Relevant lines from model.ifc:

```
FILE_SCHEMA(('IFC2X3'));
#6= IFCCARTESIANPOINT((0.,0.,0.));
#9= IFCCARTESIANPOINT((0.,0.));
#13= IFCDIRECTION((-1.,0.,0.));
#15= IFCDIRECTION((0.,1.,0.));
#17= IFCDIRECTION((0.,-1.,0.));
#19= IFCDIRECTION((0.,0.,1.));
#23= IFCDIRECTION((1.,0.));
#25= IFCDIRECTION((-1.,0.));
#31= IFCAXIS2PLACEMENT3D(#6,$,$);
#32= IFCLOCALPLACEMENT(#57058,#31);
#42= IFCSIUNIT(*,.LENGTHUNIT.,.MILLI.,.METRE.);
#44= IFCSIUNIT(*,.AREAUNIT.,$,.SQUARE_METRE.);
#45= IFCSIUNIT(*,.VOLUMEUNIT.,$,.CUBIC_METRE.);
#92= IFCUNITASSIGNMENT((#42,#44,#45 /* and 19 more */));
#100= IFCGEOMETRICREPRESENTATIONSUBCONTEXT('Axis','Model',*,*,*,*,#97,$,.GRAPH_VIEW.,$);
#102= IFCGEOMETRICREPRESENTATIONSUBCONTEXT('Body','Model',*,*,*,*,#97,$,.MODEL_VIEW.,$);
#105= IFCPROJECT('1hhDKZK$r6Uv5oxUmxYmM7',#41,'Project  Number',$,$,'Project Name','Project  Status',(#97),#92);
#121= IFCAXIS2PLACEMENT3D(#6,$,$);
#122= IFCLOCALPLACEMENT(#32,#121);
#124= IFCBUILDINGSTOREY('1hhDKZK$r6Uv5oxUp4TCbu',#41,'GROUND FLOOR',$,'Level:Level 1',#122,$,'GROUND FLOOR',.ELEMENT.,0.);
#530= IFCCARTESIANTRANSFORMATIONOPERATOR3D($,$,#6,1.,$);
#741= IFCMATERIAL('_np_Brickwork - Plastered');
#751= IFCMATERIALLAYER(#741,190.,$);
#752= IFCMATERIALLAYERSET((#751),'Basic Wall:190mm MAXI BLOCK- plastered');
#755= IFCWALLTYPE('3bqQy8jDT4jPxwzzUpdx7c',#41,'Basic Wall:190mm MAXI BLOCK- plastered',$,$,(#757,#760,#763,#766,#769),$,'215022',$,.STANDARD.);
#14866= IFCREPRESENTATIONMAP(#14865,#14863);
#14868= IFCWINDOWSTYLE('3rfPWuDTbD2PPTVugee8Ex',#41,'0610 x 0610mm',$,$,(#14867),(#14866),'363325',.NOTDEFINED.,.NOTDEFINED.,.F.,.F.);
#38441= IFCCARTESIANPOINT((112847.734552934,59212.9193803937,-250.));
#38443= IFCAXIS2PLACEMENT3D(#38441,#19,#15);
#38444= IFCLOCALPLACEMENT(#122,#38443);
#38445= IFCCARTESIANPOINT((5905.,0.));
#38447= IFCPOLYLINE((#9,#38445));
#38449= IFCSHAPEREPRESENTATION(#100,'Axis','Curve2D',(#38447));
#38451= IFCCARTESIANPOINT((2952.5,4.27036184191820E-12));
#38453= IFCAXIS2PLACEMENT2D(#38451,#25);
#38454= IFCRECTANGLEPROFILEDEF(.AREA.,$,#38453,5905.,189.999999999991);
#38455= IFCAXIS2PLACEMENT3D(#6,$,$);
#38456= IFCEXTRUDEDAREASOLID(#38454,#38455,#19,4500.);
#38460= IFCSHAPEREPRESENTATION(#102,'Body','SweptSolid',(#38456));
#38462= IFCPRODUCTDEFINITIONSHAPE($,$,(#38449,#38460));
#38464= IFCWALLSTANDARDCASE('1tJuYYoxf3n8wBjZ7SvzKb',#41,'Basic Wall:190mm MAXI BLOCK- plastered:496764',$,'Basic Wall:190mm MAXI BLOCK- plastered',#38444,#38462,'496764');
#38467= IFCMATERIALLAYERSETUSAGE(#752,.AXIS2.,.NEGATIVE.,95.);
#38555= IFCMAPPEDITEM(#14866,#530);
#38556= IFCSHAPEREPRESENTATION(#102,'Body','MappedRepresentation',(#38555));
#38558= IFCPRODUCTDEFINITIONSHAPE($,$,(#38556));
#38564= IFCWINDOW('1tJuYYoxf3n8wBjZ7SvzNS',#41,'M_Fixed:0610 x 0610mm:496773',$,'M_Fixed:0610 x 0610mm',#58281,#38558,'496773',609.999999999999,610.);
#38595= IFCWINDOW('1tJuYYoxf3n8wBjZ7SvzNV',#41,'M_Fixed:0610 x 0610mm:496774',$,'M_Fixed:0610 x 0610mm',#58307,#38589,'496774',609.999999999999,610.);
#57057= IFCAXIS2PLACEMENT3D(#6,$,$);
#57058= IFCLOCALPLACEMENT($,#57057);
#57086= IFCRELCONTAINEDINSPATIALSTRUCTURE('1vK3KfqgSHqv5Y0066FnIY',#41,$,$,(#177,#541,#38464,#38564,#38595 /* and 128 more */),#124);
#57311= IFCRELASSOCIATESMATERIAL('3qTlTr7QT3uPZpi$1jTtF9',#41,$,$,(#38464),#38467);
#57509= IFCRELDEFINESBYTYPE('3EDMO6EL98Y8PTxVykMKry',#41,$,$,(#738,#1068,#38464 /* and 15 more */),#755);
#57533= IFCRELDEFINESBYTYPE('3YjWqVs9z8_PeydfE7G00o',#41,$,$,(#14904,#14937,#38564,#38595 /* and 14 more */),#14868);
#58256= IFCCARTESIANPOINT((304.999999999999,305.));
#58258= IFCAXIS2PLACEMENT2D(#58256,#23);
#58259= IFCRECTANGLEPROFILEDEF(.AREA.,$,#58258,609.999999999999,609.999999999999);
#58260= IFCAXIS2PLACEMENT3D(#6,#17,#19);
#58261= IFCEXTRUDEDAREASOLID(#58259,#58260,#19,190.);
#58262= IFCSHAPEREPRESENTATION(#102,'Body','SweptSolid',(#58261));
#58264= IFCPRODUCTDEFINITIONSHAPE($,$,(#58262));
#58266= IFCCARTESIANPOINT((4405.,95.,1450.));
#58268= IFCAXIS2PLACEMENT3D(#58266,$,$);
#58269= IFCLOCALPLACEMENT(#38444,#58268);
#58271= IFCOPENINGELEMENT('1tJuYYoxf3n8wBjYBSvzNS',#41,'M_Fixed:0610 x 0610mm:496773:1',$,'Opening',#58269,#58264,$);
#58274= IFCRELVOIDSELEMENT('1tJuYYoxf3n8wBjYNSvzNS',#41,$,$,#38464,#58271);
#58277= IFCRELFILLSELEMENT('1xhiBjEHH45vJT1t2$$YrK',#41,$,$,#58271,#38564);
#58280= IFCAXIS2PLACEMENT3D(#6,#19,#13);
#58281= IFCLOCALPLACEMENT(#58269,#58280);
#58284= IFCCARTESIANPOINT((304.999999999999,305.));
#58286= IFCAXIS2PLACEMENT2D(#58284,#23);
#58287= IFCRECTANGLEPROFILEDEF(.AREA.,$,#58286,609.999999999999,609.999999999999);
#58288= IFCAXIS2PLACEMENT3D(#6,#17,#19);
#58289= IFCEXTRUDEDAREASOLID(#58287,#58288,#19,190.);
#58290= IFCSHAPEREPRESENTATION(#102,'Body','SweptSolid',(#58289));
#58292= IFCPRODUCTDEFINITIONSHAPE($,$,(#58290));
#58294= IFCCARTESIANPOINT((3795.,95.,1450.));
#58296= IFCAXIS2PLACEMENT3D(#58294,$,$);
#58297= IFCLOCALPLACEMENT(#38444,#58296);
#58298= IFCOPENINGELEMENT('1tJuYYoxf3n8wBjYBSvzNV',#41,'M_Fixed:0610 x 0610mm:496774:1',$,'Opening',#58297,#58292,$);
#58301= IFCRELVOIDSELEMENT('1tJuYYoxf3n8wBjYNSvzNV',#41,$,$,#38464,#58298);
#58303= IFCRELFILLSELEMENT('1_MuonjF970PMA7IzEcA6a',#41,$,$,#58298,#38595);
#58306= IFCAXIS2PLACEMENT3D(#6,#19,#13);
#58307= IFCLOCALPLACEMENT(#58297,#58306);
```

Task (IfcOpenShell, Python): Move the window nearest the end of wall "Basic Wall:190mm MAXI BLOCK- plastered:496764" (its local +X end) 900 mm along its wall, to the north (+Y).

```python
import ifcopenshell
import ifcopenshell.api.geometry
import ifcopenshell.util.placement
import ifcopenshell.util.unit

model = ifcopenshell.open("model.ifc")
unit_scale = ifcopenshell.util.unit.calculate_unit_scale(model)

window = model.by_id(38564)
opening = window.FillsVoids[0].RelatingOpeningElement
wall = opening.VoidsElements[0].RelatingBuildingElement

wall_matrix = ifcopenshell.util.placement.get_local_placement(wall.ObjectPlacement)
shift = wall_matrix[:3, 0] * 0.9 / unit_scale
before = ifcopenshell.util.placement.get_local_placement(window.ObjectPlacement)[:3, 3].copy()

# The window is placed relative to its opening, so it follows when the opening moves.
matrix = ifcopenshell.util.placement.get_local_placement(opening.ObjectPlacement)
matrix[:3, 3] += shift
ifcopenshell.api.geometry.edit_object_placement(
    model, product=opening, matrix=matrix, is_si=False, should_transform_children=True
)

after = ifcopenshell.util.placement.get_local_placement(window.ObjectPlacement)[:3, 3]
print("window moved by", (after - before).round(3) + 0.0)

model.write("model_updated.ifc")
```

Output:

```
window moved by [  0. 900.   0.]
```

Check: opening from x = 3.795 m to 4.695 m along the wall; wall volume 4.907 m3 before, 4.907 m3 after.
